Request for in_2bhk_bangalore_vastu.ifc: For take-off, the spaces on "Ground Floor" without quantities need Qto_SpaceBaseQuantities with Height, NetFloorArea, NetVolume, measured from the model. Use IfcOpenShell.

First a look at what the model holds.

```python
import ifcopenshell
import ifcopenshell.util.element
import ifcopenshell.util.unit

model = ifcopenshell.open("in_2bhk_bangalore_vastu.ifc")
print(model.schema)
for unit_type in ("LENGTHUNIT", "AREAUNIT", "VOLUMEUNIT"):
    print(unit_type, ifcopenshell.util.unit.calculate_unit_scale(model, unit_type))
storey = next(s for s in model.by_type("IfcBuildingStorey") if s.Name == "Ground Floor")
spaces = [e for e in ifcopenshell.util.element.get_decomposition(storey) if e.is_a("IfcSpace")]
for e in sorted(spaces, key=lambda e: e.id()):
    print(e.id(), e.is_a(), e.Name, list(ifcopenshell.util.element.get_psets(e, qtos_only=True)), sep=" | ")
```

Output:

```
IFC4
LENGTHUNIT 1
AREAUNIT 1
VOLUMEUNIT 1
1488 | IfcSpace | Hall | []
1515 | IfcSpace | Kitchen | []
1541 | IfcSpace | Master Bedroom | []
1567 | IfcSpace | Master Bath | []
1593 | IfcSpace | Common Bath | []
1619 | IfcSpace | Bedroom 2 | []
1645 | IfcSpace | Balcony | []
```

```python
import ifcopenshell
import ifcopenshell.api.pset
import ifcopenshell.geom
import ifcopenshell.util.element
import ifcopenshell.util.shape
import ifcopenshell.util.unit

model = ifcopenshell.open("in_2bhk_bangalore_vastu.ifc")
unit_scale = ifcopenshell.util.unit.calculate_unit_scale(model)
area_scale = ifcopenshell.util.unit.calculate_unit_scale(model, "AREAUNIT")
volume_scale = ifcopenshell.util.unit.calculate_unit_scale(model, "VOLUMEUNIT")
settings = ifcopenshell.geom.settings()

storey = next(s for s in model.by_type("IfcBuildingStorey") if s.Name == "Ground Floor")
spaces = [e for e in ifcopenshell.util.element.get_decomposition(storey) if e.is_a("IfcSpace")]

for e in sorted(spaces, key=lambda e: e.id()):
    if ifcopenshell.util.element.get_psets(e, qtos_only=True, should_inherit=False):
        continue
    # Geometry comes back in metres, in the element's own axes.
    shape = ifcopenshell.geom.create_shape(settings, e)
    values = {
        "Height": ifcopenshell.util.shape.get_z(shape.geometry) / unit_scale,
        "NetFloorArea": ifcopenshell.util.shape.get_footprint_area(shape.geometry) / area_scale,
        "NetVolume": ifcopenshell.util.shape.get_volume(shape.geometry) / volume_scale,
    }
    qto = ifcopenshell.api.pset.add_qto(model, product=e, name="Qto_SpaceBaseQuantities")
    ifcopenshell.api.pset.edit_qto(model, qto=qto, properties=values)
    print(e.id(), {k: round(v, 3) for k, v in values.items()})

model.write("in_2bhk_bangalore_vastu_v2.ifc")
```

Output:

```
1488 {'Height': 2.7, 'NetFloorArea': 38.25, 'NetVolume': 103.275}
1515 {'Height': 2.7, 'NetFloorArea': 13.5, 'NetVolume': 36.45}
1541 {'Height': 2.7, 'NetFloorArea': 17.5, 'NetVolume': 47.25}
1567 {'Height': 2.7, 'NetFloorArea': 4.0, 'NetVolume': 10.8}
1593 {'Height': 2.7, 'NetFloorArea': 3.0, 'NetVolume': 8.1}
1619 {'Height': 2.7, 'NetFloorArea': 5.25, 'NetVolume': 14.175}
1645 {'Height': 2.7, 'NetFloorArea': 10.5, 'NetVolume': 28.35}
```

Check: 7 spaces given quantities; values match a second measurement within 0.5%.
